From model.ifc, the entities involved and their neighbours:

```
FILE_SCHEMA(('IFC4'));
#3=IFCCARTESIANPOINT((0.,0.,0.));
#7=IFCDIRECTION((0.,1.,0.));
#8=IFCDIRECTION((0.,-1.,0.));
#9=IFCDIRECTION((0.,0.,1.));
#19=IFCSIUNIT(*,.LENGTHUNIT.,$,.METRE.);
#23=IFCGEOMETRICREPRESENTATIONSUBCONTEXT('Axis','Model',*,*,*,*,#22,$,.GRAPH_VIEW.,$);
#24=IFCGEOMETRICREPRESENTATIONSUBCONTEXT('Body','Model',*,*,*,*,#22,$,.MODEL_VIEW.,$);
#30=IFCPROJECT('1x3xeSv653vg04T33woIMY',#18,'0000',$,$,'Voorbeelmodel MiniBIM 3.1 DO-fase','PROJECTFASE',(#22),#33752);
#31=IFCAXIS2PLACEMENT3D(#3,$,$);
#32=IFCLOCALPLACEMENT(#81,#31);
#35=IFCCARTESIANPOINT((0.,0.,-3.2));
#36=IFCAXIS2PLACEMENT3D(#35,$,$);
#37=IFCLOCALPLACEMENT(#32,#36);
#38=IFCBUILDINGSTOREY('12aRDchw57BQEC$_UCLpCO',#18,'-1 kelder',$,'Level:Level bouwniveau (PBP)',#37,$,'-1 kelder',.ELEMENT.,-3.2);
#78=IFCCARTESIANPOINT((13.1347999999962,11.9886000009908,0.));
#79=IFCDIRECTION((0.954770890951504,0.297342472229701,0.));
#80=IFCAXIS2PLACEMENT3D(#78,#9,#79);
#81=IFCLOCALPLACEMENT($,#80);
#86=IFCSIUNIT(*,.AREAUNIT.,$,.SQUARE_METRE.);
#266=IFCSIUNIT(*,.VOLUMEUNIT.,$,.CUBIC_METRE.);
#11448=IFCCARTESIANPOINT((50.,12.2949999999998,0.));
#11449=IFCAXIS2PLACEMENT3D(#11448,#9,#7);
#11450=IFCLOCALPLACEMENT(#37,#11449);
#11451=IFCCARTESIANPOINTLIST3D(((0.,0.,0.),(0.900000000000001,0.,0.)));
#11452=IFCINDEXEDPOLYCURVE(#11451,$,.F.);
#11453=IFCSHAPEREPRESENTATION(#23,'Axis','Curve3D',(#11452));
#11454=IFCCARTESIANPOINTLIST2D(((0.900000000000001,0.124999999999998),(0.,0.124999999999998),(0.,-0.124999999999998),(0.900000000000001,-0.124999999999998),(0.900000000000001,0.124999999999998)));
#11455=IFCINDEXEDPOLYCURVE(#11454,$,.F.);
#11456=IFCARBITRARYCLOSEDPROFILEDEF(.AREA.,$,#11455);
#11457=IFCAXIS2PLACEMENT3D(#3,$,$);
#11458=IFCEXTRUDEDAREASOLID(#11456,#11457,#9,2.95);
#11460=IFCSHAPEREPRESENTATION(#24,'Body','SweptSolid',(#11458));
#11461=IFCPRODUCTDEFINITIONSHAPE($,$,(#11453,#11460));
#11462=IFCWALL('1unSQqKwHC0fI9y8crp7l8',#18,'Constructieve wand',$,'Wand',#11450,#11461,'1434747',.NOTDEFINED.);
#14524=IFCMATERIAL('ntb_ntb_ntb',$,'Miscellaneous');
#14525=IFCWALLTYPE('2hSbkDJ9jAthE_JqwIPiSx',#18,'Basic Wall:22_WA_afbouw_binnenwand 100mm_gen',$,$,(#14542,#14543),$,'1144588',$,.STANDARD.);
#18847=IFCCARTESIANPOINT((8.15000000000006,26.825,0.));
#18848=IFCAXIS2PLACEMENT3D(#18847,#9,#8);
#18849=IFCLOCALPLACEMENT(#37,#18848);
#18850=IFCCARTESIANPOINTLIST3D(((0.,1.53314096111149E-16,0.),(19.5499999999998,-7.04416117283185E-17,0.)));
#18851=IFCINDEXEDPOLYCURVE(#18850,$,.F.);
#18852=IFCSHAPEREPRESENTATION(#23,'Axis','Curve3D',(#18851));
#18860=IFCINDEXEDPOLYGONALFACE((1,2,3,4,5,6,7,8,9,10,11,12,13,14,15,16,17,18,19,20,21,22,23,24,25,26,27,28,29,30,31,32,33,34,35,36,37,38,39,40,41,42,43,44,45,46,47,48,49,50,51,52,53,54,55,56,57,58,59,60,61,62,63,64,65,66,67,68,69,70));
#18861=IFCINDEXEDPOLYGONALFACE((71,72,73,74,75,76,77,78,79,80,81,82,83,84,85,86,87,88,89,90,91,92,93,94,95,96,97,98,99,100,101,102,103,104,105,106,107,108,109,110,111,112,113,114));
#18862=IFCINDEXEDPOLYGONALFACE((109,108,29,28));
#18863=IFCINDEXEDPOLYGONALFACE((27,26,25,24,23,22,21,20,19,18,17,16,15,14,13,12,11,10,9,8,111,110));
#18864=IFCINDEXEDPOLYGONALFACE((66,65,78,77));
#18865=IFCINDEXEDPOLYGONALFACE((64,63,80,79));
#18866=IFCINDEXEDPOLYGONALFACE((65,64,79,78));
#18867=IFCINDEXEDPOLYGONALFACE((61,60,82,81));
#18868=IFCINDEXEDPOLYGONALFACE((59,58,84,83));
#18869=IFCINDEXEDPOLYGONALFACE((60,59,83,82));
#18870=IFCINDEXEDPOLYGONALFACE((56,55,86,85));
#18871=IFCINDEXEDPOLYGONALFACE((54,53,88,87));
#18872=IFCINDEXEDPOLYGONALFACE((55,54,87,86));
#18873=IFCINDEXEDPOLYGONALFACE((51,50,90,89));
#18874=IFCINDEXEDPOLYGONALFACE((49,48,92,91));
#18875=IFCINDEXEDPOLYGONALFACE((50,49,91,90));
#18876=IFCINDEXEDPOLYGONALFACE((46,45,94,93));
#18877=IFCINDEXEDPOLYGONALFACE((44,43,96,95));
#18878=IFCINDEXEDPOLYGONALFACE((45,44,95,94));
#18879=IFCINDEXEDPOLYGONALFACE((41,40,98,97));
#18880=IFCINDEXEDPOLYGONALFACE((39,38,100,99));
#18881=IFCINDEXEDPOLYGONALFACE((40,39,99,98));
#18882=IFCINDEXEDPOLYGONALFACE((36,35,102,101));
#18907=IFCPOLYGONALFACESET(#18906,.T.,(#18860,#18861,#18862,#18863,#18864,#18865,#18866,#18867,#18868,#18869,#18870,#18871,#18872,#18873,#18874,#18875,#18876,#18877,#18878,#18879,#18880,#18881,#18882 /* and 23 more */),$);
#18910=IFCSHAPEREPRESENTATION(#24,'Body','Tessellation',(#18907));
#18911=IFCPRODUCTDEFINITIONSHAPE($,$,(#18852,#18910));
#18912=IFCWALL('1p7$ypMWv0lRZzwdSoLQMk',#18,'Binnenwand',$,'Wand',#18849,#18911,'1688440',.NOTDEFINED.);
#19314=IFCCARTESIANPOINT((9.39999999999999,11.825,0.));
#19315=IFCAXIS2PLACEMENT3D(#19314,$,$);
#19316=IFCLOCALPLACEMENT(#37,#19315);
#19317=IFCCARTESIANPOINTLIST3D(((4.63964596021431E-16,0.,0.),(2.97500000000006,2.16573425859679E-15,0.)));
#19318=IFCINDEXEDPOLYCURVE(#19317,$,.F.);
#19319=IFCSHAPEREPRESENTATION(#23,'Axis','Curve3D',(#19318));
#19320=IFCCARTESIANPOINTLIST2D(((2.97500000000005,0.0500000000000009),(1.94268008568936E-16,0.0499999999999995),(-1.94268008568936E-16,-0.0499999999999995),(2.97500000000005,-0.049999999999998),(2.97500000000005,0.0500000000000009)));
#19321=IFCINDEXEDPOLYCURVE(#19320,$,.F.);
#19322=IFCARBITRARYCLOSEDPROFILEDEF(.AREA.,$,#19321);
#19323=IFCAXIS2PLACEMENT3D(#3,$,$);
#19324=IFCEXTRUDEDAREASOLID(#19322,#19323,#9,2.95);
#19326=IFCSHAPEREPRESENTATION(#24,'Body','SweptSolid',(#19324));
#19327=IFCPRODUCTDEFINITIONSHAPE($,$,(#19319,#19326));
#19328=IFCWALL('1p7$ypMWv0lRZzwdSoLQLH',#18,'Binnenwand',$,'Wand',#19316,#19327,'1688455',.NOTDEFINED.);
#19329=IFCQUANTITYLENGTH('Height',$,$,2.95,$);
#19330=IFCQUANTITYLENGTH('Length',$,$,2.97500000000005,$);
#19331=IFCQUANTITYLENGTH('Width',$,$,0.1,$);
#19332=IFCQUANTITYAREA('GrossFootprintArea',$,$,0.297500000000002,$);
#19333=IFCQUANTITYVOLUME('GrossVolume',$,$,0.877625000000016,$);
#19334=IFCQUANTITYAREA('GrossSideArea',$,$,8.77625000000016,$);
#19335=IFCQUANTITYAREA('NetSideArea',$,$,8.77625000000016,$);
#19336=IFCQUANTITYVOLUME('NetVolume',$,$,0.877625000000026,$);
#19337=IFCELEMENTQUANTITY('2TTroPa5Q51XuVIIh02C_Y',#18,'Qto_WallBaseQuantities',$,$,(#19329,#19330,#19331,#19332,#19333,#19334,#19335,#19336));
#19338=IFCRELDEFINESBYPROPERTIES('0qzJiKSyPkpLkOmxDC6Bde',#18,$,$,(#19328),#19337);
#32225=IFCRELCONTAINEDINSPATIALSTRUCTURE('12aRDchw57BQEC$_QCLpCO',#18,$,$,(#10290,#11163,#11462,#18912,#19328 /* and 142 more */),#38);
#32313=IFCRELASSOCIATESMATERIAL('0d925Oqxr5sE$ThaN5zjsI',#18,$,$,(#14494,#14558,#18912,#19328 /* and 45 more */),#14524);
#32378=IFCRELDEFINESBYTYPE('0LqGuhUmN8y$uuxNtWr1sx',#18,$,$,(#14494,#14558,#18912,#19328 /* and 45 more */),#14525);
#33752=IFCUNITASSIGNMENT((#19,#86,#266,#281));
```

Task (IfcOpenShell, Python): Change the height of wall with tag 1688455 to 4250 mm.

```python
import ifcopenshell
import ifcopenshell.api.pset
import ifcopenshell.geom
import ifcopenshell.util.element
import ifcopenshell.util.representation
import ifcopenshell.util.shape
import ifcopenshell.util.unit

model = ifcopenshell.open("model.ifc")
unit_scale = ifcopenshell.util.unit.calculate_unit_scale(model)
area_scale = ifcopenshell.util.unit.calculate_unit_scale(model, "AREAUNIT")
volume_scale = ifcopenshell.util.unit.calculate_unit_scale(model, "VOLUMEUNIT")
settings = ifcopenshell.geom.settings()


def volume(element):
    """Net volume in cubic metres, openings subtracted."""
    shape = ifcopenshell.geom.create_shape(settings, element)
    return ifcopenshell.util.shape.get_volume(shape.geometry)


wall = model.by_id(19328)
before = volume(wall)

body = ifcopenshell.util.representation.get_representation(wall, "Model", "Body")
solid = body.Items[0]
old_height = solid.Depth
solid.Depth = 4.25 / unit_scale
after = volume(wall)
thickness = 0.1  # wall thickness in metres

# Update the stored height, areas and volumes.
qto = model.by_id(ifcopenshell.util.element.get_pset(wall, "Qto_WallBaseQuantities", should_inherit=False)["id"])
ifcopenshell.api.pset.edit_qto(model, qto=qto, properties={
    "Height": solid.Depth,
    "GrossVolume": ifcopenshell.util.element.get_pset(wall, "Qto_WallBaseQuantities", "GrossVolume") * solid.Depth / old_height,
    "GrossSideArea": ifcopenshell.util.element.get_pset(wall, "Qto_WallBaseQuantities", "GrossSideArea") * solid.Depth / old_height,
    "NetSideArea": after / thickness / area_scale,
    "NetVolume": after / volume_scale,
})

print(f"height {old_height:g} -> {solid.Depth:g}, volume {before:.3f} -> {after:.3f} m3")

model.write("model_v2.ifc")
```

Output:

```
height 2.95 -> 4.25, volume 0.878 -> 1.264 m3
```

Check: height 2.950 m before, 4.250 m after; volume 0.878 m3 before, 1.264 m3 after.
